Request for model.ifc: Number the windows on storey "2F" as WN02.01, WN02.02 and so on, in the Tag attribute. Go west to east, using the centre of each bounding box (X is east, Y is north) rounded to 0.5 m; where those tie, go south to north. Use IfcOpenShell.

First a look at what the model holds.

```python
import ifcopenshell
import ifcopenshell.util.element
import ifcopenshell.util.placement

model = ifcopenshell.open("model.ifc")
print(model.schema)
storey = next(s for s in model.by_type("IfcBuildingStorey") if s.Name == "2F")
windows = [e for e in ifcopenshell.util.element.get_decomposition(storey) if e.is_a("IfcWindow")]
for e in sorted(windows, key=lambda e: e.id()):
    origin = ifcopenshell.util.placement.get_local_placement(e.ObjectPlacement)[:3, 3]
    print(e.id(), e.Tag, e.Name, origin.round(2) + 0.0, sep=" | ")
```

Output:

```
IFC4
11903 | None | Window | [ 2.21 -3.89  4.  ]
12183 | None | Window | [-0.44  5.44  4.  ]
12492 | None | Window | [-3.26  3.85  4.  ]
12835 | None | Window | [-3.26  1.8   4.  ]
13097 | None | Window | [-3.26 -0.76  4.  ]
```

```python
import ifcopenshell
import ifcopenshell.geom
import ifcopenshell.util.element
import ifcopenshell.util.shape

model = ifcopenshell.open("model.ifc")
settings = ifcopenshell.geom.settings()
settings.set("use-world-coords", True)


def centre(element):
    shape = ifcopenshell.geom.create_shape(settings, element)
    return ifcopenshell.util.shape.get_bbox_centroid(shape.geometry)


storey = next(s for s in model.by_type("IfcBuildingStorey") if s.Name == "2F")
windows = [e for e in ifcopenshell.util.element.get_decomposition(storey) if e.is_a("IfcWindow")]

# Insertion points can sit at a corner or the storey origin, so sort by the geometry (in metres).
centres = {e: centre(e) for e in windows}
windows.sort(key=lambda e: (round(centres[e][0] / 0.5), centres[e][1]))

for i, e in enumerate(windows, start=1):
    number = f"WN02.{i:02d}"
    e.Tag = number
    print(e.id(), number)

model.write("model_updated.ifc")
```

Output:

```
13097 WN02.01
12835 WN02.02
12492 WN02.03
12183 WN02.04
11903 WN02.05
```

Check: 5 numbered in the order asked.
